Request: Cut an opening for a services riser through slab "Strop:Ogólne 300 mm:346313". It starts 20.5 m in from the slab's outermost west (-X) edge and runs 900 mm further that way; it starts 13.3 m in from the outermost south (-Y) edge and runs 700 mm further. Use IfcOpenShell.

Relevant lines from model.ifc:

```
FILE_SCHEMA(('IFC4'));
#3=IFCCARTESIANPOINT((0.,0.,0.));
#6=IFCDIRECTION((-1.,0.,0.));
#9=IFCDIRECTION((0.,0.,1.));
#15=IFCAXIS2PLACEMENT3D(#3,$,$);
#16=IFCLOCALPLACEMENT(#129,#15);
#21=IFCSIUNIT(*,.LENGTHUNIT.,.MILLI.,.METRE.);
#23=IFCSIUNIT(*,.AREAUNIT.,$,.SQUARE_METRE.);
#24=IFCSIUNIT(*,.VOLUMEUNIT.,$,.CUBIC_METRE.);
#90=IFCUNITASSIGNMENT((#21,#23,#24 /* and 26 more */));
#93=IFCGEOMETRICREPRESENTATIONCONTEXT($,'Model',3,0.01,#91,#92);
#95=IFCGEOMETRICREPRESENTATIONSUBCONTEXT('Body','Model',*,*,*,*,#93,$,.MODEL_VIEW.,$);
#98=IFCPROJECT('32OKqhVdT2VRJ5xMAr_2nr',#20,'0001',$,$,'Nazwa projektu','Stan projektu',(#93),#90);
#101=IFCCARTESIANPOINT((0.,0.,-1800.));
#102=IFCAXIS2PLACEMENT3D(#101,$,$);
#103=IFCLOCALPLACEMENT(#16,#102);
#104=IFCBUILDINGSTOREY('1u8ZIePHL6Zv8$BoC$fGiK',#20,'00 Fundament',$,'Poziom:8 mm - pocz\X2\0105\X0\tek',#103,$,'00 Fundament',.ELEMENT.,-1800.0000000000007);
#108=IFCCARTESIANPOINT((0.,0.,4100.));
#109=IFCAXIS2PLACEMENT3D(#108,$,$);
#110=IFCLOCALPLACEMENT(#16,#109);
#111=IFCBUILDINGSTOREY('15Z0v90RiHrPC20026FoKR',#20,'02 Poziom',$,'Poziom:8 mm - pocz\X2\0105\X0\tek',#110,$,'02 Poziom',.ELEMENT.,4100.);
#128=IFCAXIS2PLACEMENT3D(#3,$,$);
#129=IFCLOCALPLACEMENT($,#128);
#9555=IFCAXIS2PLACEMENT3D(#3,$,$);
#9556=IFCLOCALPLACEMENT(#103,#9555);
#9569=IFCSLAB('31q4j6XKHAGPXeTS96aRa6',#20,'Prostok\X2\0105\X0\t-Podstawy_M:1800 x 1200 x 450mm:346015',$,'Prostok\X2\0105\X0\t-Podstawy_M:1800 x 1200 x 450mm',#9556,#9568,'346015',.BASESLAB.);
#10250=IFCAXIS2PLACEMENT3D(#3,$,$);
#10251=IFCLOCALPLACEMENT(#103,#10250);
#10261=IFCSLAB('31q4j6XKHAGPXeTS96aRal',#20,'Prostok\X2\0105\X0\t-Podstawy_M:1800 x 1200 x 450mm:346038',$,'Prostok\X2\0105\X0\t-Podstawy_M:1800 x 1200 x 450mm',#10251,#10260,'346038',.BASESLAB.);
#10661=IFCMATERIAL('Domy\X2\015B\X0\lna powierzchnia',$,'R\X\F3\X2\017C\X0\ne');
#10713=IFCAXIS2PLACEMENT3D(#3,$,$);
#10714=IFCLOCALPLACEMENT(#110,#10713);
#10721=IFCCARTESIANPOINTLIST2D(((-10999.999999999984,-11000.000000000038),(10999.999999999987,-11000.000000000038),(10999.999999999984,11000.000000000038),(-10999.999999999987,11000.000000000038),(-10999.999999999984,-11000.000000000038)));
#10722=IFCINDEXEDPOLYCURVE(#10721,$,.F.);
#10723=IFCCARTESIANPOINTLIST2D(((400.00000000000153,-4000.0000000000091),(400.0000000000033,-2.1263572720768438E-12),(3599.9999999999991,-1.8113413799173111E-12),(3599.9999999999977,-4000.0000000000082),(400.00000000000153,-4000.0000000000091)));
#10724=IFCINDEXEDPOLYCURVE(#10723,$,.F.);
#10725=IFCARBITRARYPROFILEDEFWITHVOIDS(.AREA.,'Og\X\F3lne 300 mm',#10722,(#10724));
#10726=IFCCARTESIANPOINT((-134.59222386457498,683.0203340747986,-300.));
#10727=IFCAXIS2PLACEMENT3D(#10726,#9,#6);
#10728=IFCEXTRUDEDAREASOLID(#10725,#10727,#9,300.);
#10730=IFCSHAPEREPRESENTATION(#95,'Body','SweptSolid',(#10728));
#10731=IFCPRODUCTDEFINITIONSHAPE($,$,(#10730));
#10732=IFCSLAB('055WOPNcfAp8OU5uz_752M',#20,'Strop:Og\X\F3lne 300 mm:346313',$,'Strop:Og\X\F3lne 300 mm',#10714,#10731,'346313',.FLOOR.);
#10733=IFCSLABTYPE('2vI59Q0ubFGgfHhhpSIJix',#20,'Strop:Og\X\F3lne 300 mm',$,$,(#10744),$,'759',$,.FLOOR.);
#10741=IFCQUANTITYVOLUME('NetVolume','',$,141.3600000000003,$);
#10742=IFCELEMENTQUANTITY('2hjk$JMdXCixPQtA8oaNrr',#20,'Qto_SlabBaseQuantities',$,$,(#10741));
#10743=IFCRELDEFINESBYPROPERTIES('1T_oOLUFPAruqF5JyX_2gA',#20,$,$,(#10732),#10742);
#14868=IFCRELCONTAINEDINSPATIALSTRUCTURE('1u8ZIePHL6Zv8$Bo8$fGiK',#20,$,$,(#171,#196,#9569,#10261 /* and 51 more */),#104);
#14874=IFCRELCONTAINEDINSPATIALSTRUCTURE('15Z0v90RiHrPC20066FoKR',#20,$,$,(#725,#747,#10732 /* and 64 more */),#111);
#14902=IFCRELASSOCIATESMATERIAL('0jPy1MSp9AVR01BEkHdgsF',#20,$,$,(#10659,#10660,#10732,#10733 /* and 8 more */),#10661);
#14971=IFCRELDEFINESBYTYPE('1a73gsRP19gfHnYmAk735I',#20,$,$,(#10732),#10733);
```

```python
import numpy as np
import ifcopenshell
import ifcopenshell.api.feature
import ifcopenshell.api.geometry
import ifcopenshell.api.pset
import ifcopenshell.api.root
import ifcopenshell.geom
import ifcopenshell.util.element
import ifcopenshell.util.placement
import ifcopenshell.util.representation
import ifcopenshell.util.shape
import ifcopenshell.util.unit

model = ifcopenshell.open("model.ifc")
unit_scale = ifcopenshell.util.unit.calculate_unit_scale(model)
volume_scale = ifcopenshell.util.unit.calculate_unit_scale(model, "VOLUMEUNIT")
settings = ifcopenshell.geom.settings()


def volume(element):
    """Net volume in cubic metres, openings subtracted."""
    shape = ifcopenshell.geom.create_shape(settings, element)
    return ifcopenshell.util.shape.get_volume(shape.geometry)


slab = model.by_guid("055WOPNcfAp8OU5uz_752M")
before = volume(slab)

# Extent in the slab's own axes, in metres. The edges named are its -X and -Y sides.
slab_shape = ifcopenshell.geom.create_shape(settings, slab)
vertices = ifcopenshell.util.shape.get_vertices(slab_shape.geometry)
x_min, y_min, bottom = vertices.min(axis=0)
top = vertices[:, 2].max()

opening = ifcopenshell.api.root.create_entity(model, ifc_class="IfcOpeningElement", name="Services riser opening", predefined_type="OPENING")
context = ifcopenshell.util.representation.get_context(model, "Model", "Body", "MODEL_VIEW")
width, depth = 0.9, 0.7
outline = [(0.0, 0.0), (width, 0.0), (width, depth), (0.0, depth), (0.0, 0.0)]
# Overshoot both faces by 50 mm so the cut is clean.
shape = ifcopenshell.api.geometry.add_slab_representation(
    model, context=context, depth=top - bottom + 0.1, polyline=outline
)
ifcopenshell.api.geometry.assign_representation(model, product=opening, representation=shape)

matrix = ifcopenshell.util.placement.get_local_placement(slab.ObjectPlacement)
matrix[:, 3] = matrix @ np.append(np.array([x_min + 20.5, y_min + 13.3, bottom - 0.05]) / unit_scale, 1.0)
ifcopenshell.api.geometry.edit_object_placement(model, product=opening, matrix=matrix, is_si=False)
ifcopenshell.api.feature.add_feature(model, feature=opening, element=slab)

after = volume(slab)

# Update the slab's stored quantities.
qto = model.by_id(ifcopenshell.util.element.get_pset(slab, "Qto_SlabBaseQuantities", should_inherit=False)["id"])
ifcopenshell.api.pset.edit_qto(model, qto=qto, properties={"NetVolume": after / volume_scale})

print(f"slab volume {before:.3f} -> {after:.3f} m3")

model.write("model_rev.ifc")
```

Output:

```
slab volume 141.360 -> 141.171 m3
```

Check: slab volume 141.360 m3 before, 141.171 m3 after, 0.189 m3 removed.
